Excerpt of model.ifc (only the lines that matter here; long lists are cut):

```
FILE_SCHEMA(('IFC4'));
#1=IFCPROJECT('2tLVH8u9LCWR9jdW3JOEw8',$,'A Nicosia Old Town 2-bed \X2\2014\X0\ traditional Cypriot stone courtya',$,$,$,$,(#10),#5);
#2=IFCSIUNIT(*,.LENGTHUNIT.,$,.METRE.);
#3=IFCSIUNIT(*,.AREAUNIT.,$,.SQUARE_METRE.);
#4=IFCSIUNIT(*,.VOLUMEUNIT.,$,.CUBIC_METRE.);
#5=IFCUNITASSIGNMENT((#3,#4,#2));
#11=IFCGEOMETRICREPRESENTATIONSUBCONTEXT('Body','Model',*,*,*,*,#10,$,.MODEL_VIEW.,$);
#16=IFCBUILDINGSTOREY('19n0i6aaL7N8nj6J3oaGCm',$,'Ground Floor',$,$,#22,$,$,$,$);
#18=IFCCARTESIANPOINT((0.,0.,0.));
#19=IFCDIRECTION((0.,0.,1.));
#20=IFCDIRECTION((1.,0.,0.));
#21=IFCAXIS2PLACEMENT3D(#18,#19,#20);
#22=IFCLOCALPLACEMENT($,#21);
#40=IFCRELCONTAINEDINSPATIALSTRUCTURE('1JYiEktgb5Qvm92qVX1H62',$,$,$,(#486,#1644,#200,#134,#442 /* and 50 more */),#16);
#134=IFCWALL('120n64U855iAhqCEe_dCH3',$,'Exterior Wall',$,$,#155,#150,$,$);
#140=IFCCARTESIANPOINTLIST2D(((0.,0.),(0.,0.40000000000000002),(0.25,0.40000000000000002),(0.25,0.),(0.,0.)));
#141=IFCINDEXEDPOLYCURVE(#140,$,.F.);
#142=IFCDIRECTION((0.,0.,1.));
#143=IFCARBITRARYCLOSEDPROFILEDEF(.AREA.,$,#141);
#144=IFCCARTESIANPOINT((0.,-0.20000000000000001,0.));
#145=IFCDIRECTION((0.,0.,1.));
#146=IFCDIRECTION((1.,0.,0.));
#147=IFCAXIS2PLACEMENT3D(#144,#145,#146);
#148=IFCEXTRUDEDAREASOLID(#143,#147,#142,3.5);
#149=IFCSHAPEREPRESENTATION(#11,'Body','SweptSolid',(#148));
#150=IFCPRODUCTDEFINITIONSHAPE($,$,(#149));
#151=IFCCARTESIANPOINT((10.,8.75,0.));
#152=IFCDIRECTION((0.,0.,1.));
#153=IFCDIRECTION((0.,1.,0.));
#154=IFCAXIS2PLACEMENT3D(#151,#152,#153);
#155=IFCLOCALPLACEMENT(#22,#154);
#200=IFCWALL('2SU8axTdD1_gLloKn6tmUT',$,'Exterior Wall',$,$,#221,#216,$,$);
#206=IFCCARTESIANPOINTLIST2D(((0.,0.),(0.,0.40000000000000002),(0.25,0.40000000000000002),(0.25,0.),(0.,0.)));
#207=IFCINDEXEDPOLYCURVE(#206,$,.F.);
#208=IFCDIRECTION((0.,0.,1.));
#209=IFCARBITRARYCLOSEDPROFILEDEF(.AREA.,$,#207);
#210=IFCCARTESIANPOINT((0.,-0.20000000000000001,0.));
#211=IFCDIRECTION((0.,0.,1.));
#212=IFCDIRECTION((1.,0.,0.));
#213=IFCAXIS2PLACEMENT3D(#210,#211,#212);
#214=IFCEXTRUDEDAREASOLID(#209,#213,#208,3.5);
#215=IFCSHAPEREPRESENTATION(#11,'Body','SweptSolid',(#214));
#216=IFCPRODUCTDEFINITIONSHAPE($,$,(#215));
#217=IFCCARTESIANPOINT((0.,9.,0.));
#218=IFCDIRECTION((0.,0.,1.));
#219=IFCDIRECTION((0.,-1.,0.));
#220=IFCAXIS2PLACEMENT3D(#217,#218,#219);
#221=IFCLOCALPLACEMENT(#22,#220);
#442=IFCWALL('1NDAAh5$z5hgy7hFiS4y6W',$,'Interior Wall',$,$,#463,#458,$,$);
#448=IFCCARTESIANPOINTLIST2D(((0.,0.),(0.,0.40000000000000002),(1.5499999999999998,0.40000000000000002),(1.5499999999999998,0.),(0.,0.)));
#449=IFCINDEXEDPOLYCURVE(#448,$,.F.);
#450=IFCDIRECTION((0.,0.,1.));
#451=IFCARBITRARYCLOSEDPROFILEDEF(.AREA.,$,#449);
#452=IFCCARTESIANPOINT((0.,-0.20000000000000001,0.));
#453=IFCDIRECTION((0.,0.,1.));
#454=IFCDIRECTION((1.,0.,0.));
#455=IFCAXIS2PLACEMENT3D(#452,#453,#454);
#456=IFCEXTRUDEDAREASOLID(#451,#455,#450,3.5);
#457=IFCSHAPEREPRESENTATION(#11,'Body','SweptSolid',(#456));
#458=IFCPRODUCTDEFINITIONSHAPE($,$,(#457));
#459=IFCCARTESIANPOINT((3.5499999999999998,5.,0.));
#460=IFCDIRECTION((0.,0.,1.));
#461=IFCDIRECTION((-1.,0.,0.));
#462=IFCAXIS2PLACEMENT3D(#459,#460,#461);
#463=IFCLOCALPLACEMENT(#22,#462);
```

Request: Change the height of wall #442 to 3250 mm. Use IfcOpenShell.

```python
import ifcopenshell
import ifcopenshell.geom
import ifcopenshell.util.representation
import ifcopenshell.util.shape

model = ifcopenshell.open("model.ifc")
settings = ifcopenshell.geom.settings()


def volume(element):
    """Net volume in cubic metres, openings subtracted."""
    shape = ifcopenshell.geom.create_shape(settings, element)
    return ifcopenshell.util.shape.get_volume(shape.geometry)


wall = model.by_guid("1NDAAh5$z5hgy7hFiS4y6W")
before = volume(wall)

body = ifcopenshell.util.representation.get_representation(wall, "Model", "Body")
solid = body.Items[0]
old_height = solid.Depth
solid.Depth = 3.25
after = volume(wall)

print(f"height {old_height:g} -> {solid.Depth:g}, volume {before:.3f} -> {after:.3f} m3")

model.write("model_rev.ifc")
```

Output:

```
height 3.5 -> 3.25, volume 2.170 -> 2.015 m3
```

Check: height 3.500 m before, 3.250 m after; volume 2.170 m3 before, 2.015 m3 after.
